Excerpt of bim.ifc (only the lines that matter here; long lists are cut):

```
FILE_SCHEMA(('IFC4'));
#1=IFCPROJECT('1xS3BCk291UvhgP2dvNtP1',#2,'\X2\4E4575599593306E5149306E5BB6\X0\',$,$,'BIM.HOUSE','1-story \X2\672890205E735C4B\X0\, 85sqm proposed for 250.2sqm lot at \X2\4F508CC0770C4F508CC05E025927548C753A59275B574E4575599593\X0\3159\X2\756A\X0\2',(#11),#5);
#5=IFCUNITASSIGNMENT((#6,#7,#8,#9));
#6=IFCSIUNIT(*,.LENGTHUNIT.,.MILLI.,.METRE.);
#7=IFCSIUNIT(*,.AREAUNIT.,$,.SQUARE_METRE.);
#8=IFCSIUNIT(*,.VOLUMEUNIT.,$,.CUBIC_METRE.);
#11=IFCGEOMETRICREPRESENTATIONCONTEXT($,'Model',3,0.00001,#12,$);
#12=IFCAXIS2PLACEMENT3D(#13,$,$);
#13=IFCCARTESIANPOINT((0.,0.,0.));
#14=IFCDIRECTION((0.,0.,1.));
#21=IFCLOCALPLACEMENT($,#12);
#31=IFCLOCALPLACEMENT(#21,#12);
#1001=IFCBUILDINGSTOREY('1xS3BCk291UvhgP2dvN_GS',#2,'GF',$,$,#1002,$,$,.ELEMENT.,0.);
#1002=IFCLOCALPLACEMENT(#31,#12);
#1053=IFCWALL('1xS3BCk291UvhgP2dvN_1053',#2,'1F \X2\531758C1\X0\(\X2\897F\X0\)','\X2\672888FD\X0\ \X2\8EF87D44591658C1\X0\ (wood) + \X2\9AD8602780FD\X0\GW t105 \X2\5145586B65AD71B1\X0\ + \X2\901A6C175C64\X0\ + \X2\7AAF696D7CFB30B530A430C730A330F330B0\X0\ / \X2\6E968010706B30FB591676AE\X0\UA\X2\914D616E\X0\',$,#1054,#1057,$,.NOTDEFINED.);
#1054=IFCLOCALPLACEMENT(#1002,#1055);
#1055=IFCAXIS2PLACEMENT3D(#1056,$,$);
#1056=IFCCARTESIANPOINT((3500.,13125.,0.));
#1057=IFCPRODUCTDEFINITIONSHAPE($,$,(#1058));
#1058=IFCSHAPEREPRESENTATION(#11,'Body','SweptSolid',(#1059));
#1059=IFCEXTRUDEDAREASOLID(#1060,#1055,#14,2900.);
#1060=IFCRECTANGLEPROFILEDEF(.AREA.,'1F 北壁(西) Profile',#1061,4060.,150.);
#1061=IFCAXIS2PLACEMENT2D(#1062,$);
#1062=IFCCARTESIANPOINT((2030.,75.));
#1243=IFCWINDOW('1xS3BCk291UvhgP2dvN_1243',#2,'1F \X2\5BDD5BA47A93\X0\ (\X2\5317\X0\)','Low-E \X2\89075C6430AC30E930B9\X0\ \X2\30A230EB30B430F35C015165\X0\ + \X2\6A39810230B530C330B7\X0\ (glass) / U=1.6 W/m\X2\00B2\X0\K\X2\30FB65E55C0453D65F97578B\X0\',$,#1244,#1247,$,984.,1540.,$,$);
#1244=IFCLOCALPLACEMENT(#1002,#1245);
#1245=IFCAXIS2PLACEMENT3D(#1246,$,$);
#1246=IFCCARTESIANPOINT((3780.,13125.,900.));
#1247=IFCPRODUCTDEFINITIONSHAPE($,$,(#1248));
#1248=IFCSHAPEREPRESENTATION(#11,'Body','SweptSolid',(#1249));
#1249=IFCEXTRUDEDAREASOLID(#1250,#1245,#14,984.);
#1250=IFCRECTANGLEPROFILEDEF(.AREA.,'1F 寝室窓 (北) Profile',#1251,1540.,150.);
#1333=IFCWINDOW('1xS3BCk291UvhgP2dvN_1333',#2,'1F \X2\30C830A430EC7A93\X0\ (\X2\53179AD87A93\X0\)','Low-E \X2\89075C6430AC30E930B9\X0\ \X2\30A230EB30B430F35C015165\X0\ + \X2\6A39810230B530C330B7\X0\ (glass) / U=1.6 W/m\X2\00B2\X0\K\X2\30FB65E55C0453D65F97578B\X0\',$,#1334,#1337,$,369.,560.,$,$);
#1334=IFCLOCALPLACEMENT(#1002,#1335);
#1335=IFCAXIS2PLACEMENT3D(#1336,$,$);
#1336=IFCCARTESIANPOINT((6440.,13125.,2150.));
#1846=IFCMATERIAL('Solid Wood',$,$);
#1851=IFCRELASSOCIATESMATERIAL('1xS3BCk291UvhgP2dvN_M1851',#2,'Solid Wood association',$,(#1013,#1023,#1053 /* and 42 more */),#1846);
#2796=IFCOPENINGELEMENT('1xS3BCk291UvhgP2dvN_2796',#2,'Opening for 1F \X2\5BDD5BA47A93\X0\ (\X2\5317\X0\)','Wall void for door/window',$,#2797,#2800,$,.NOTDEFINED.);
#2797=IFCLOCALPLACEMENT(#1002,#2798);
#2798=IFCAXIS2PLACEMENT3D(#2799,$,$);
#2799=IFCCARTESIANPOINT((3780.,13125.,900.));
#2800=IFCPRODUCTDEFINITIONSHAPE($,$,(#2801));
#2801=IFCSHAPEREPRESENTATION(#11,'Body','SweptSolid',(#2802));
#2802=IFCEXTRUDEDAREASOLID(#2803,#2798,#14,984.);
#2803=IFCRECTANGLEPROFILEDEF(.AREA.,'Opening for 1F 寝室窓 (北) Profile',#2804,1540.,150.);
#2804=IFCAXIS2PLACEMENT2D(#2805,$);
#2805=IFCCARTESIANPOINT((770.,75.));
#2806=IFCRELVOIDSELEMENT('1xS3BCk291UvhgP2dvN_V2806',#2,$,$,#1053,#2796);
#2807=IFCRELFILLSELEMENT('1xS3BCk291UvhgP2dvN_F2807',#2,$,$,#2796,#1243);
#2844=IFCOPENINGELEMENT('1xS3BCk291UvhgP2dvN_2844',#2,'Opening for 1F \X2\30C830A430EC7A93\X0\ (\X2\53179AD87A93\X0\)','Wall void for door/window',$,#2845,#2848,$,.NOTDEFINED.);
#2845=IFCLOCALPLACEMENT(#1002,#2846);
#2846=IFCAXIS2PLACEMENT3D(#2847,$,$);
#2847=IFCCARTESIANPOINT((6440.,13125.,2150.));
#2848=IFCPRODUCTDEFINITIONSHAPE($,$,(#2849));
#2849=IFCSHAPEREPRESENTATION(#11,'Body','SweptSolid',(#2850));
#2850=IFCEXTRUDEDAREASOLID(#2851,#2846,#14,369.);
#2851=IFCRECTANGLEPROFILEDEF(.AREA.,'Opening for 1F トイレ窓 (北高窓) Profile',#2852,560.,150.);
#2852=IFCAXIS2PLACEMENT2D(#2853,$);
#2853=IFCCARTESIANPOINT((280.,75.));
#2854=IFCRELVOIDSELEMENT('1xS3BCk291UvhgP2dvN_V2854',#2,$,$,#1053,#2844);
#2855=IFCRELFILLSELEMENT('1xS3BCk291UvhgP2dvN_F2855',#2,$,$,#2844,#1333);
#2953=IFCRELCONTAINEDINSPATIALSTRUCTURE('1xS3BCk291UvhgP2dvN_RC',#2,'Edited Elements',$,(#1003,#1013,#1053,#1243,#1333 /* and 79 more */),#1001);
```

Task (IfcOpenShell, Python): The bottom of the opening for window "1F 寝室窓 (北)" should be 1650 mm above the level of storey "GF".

```python
import numpy as np
import ifcopenshell
import ifcopenshell.api.geometry
import ifcopenshell.geom
import ifcopenshell.util.element
import ifcopenshell.util.placement
import ifcopenshell.util.shape
import ifcopenshell.util.unit

model = ifcopenshell.open("bim.ifc")
unit_scale = ifcopenshell.util.unit.calculate_unit_scale(model)

window = model.by_id(1243)
opening = window.FillsVoids[0].RelatingOpeningElement
storey = ifcopenshell.util.element.get_container(window, ifc_class="IfcBuildingStorey")
level = ifcopenshell.util.placement.get_local_placement(storey.ObjectPlacement)[2, 3]

# The opening's origin need not be at the sill, so measure its lowest point.
shape = ifcopenshell.geom.create_shape(ifcopenshell.geom.settings(), opening)
bottom = ifcopenshell.util.shape.get_shape_bottom_elevation(shape, shape.geometry) / unit_scale
dz = level + 1.65 / unit_scale - bottom

shift = np.array([0.0, 0.0, dz])
# The window is not placed relative to its opening, so move both.
for product in (opening, window):
    matrix = ifcopenshell.util.placement.get_local_placement(product.ObjectPlacement)
    matrix[:3, 3] += shift
    ifcopenshell.api.geometry.edit_object_placement(model, product=product, matrix=matrix, is_si=False)

print(f"moved by {dz * unit_scale:+.3f} m")

model.write("bim_updated.ifc")
```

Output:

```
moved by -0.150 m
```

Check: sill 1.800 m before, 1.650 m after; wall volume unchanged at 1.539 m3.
